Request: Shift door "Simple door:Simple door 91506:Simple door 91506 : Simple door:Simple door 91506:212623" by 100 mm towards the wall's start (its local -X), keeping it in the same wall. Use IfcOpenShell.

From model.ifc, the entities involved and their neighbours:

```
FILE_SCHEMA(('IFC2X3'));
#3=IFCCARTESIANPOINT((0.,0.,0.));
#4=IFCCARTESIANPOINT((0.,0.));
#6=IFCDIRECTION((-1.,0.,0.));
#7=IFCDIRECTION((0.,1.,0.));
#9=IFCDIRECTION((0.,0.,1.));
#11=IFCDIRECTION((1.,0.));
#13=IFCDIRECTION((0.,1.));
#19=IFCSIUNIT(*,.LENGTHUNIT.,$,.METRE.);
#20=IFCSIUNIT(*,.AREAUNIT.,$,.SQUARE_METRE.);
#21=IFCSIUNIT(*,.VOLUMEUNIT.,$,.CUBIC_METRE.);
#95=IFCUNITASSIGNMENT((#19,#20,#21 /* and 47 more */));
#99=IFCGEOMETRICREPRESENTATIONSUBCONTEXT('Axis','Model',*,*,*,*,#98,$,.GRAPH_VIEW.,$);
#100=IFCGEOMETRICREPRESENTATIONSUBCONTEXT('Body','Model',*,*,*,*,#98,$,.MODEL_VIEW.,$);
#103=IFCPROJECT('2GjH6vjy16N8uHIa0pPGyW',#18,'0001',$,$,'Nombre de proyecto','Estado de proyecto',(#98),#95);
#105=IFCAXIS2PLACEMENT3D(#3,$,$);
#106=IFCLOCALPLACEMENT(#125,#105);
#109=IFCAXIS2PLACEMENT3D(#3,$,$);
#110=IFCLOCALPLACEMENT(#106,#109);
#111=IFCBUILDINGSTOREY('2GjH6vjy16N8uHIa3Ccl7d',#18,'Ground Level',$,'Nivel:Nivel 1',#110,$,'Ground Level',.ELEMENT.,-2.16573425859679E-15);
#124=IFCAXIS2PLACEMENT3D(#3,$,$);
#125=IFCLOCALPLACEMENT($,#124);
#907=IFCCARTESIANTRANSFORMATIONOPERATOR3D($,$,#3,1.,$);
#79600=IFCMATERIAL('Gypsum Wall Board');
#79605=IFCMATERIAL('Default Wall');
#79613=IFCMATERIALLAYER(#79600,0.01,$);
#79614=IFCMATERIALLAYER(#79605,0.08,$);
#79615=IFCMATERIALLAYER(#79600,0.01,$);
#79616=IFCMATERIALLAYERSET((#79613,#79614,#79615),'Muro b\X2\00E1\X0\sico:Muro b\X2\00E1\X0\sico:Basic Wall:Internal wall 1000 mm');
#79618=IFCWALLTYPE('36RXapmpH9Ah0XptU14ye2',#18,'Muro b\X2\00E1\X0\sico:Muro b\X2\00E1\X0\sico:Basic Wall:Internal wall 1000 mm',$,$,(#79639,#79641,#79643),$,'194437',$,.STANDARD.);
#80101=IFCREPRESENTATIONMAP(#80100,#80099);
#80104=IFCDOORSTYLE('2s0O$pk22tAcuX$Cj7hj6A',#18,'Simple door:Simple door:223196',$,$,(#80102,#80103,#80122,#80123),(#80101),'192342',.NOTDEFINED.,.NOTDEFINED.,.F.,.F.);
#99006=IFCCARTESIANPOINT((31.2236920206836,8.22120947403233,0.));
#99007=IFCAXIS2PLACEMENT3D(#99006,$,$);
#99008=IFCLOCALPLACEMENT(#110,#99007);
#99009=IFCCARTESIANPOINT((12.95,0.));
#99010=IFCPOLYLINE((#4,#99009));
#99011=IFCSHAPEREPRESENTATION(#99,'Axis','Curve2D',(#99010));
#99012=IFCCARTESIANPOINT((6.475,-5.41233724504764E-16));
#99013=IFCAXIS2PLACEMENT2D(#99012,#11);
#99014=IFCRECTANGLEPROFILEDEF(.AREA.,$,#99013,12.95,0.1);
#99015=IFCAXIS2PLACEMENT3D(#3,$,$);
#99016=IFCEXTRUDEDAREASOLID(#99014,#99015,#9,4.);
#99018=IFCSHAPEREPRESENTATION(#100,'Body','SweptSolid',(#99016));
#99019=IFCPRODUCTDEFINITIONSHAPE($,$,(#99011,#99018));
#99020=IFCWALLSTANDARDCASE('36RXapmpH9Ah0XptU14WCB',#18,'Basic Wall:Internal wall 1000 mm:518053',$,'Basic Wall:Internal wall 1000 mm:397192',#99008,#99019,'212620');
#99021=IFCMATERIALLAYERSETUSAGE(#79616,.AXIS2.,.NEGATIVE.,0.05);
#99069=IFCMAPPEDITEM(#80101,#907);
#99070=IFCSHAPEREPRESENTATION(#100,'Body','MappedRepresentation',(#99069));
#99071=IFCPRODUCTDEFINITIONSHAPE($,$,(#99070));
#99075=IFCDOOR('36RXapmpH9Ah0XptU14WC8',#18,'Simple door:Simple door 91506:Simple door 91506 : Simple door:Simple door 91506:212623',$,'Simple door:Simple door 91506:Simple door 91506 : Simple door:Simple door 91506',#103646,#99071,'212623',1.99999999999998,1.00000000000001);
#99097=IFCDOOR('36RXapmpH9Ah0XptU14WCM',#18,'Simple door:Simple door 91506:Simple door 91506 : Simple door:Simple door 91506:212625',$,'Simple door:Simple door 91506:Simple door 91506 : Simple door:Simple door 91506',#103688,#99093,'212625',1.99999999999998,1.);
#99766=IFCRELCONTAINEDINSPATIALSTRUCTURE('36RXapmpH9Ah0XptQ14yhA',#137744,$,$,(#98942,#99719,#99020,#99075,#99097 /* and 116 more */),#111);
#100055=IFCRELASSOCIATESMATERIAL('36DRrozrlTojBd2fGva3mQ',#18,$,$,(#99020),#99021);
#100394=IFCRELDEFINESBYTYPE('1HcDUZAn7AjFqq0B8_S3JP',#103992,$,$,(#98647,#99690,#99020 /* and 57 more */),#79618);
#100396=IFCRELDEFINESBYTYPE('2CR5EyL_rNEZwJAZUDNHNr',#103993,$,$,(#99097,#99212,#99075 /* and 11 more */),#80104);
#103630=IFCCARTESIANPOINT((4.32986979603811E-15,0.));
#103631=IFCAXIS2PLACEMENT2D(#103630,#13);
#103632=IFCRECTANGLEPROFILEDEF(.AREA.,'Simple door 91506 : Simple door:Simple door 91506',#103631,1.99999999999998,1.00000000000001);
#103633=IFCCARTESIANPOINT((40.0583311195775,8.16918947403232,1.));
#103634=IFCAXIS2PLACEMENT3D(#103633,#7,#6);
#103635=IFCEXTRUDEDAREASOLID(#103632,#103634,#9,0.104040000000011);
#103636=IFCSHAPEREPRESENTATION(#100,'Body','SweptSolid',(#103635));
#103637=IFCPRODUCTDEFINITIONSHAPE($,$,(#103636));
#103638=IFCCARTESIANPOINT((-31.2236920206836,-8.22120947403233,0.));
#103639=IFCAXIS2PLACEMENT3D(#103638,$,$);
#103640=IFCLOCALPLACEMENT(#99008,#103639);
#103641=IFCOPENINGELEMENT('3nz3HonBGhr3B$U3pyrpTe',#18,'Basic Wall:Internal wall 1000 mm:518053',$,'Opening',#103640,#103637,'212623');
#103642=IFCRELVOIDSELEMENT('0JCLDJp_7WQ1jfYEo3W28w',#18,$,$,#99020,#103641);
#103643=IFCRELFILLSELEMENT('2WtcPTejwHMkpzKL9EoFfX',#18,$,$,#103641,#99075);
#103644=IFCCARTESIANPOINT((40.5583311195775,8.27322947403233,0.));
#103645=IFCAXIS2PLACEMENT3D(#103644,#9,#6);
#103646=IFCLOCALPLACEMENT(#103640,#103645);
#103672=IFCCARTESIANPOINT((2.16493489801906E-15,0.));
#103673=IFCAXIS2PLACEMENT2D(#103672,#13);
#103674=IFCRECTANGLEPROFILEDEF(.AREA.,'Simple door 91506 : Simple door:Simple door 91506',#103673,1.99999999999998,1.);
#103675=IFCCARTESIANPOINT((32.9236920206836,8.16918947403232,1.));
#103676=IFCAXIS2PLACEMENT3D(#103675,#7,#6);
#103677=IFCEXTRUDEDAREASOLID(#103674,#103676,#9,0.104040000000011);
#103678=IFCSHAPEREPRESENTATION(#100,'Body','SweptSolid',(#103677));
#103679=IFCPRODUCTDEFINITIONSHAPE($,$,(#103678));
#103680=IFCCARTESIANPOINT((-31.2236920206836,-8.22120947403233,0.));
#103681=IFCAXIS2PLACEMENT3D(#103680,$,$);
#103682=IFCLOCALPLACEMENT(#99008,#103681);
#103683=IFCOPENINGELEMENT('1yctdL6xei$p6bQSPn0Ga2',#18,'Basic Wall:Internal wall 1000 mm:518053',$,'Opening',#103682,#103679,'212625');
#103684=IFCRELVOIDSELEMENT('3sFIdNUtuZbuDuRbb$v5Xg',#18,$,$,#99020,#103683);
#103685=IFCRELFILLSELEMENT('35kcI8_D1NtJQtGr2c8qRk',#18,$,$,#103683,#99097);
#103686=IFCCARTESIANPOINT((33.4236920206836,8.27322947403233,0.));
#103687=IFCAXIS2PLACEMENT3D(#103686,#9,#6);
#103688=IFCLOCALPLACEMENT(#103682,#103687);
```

```python
import ifcopenshell
import ifcopenshell.api.geometry
import ifcopenshell.util.placement
import ifcopenshell.util.unit

model = ifcopenshell.open("model.ifc")
unit_scale = ifcopenshell.util.unit.calculate_unit_scale(model)

door = model.by_guid("36RXapmpH9Ah0XptU14WC8")
opening = door.FillsVoids[0].RelatingOpeningElement
wall = opening.VoidsElements[0].RelatingBuildingElement

wall_matrix = ifcopenshell.util.placement.get_local_placement(wall.ObjectPlacement)
shift = wall_matrix[:3, 0] * -0.1 / unit_scale
before = ifcopenshell.util.placement.get_local_placement(door.ObjectPlacement)[:3, 3].copy()

# The door is placed relative to its opening, so it follows when the opening moves.
matrix = ifcopenshell.util.placement.get_local_placement(opening.ObjectPlacement)
matrix[:3, 3] += shift
ifcopenshell.api.geometry.edit_object_placement(
    model, product=opening, matrix=matrix, is_si=False, should_transform_children=True
)

after = ifcopenshell.util.placement.get_local_placement(door.ObjectPlacement)[:3, 3]
print("door moved by", (after - before).round(3) + 0.0)

model.write("model_rev.ifc")
```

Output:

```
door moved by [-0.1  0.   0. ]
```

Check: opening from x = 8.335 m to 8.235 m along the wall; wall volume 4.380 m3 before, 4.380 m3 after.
